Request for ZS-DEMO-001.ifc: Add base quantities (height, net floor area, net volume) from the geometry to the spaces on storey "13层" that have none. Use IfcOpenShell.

First a look at what the model holds.

```python
import ifcopenshell
import ifcopenshell.util.element
import ifcopenshell.util.unit

model = ifcopenshell.open("ZS-DEMO-001.ifc")
print(model.schema)
for unit_type in ("LENGTHUNIT", "AREAUNIT", "VOLUMEUNIT"):
    print(unit_type, ifcopenshell.util.unit.calculate_unit_scale(model, unit_type))
storey = next(s for s in model.by_type("IfcBuildingStorey") if s.Name == "13层")
spaces = [e for e in ifcopenshell.util.element.get_decomposition(storey) if e.is_a("IfcSpace")]
for e in sorted(spaces, key=lambda e: e.id()):
    print(e.id(), e.is_a(), e.Name, list(ifcopenshell.util.element.get_psets(e, qtos_only=True)), sep=" | ")
```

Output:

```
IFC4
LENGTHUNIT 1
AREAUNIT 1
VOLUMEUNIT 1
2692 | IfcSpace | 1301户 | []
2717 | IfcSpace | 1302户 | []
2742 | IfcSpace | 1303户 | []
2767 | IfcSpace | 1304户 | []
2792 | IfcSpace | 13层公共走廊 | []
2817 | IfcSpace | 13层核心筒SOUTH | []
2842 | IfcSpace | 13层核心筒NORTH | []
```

```python
import ifcopenshell
import ifcopenshell.api.pset
import ifcopenshell.geom
import ifcopenshell.util.element
import ifcopenshell.util.shape
import ifcopenshell.util.unit

model = ifcopenshell.open("ZS-DEMO-001.ifc")
unit_scale = ifcopenshell.util.unit.calculate_unit_scale(model)
area_scale = ifcopenshell.util.unit.calculate_unit_scale(model, "AREAUNIT")
volume_scale = ifcopenshell.util.unit.calculate_unit_scale(model, "VOLUMEUNIT")
settings = ifcopenshell.geom.settings()

storey = next(s for s in model.by_type("IfcBuildingStorey") if s.Name == "13层")
spaces = [e for e in ifcopenshell.util.element.get_decomposition(storey) if e.is_a("IfcSpace")]

for e in sorted(spaces, key=lambda e: e.id()):
    if ifcopenshell.util.element.get_psets(e, qtos_only=True, should_inherit=False):
        continue
    # Geometry comes back in metres, in the element's own axes.
    shape = ifcopenshell.geom.create_shape(settings, e)
    values = {
        "Height": ifcopenshell.util.shape.get_z(shape.geometry) / unit_scale,
        "NetFloorArea": ifcopenshell.util.shape.get_footprint_area(shape.geometry) / area_scale,
        "NetVolume": ifcopenshell.util.shape.get_volume(shape.geometry) / volume_scale,
    }
    qto = ifcopenshell.api.pset.add_qto(model, product=e, name="Qto_SpaceBaseQuantities")
    ifcopenshell.api.pset.edit_qto(model, qto=qto, properties=values)
    print(e.id(), {k: round(v, 3) for k, v in values.items()})

model.write("ZS-DEMO-001_rev.ifc")
```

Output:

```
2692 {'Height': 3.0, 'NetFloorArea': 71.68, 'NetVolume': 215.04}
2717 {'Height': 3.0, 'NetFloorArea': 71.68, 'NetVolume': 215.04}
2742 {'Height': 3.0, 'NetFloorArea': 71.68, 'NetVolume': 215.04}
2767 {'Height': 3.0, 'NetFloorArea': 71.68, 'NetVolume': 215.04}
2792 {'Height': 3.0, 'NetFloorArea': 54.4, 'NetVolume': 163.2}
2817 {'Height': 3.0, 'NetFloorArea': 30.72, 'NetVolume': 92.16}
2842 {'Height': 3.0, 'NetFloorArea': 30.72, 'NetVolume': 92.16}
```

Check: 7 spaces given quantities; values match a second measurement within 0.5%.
